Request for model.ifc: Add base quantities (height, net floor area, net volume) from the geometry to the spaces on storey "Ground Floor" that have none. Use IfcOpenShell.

First a look at what the model holds.

```python
import ifcopenshell
import ifcopenshell.util.element
import ifcopenshell.util.unit

model = ifcopenshell.open("model.ifc")
print(model.schema)
for unit_type in ("LENGTHUNIT", "AREAUNIT", "VOLUMEUNIT"):
    print(unit_type, ifcopenshell.util.unit.calculate_unit_scale(model, unit_type))
storey = next(s for s in model.by_type("IfcBuildingStorey") if s.Name == "Ground Floor")
spaces = [e for e in ifcopenshell.util.element.get_decomposition(storey) if e.is_a("IfcSpace")]
for e in sorted(spaces, key=lambda e: e.id()):
    print(e.id(), e.is_a(), e.Name, list(ifcopenshell.util.element.get_psets(e, qtos_only=True)), sep=" | ")
```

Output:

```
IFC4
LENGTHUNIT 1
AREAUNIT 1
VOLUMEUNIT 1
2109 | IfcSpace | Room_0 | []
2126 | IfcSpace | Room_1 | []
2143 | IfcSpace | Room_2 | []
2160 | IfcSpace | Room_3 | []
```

```python
import ifcopenshell
import ifcopenshell.api.pset
import ifcopenshell.geom
import ifcopenshell.util.element
import ifcopenshell.util.shape
import ifcopenshell.util.unit

model = ifcopenshell.open("model.ifc")
unit_scale = ifcopenshell.util.unit.calculate_unit_scale(model)
area_scale = ifcopenshell.util.unit.calculate_unit_scale(model, "AREAUNIT")
volume_scale = ifcopenshell.util.unit.calculate_unit_scale(model, "VOLUMEUNIT")
settings = ifcopenshell.geom.settings()

storey = next(s for s in model.by_type("IfcBuildingStorey") if s.Name == "Ground Floor")
spaces = [e for e in ifcopenshell.util.element.get_decomposition(storey) if e.is_a("IfcSpace")]

for e in sorted(spaces, key=lambda e: e.id()):
    if ifcopenshell.util.element.get_psets(e, qtos_only=True, should_inherit=False):
        continue
    # Geometry comes back in metres, in the element's own axes.
    shape = ifcopenshell.geom.create_shape(settings, e)
    values = {
        "Height": ifcopenshell.util.shape.get_z(shape.geometry) / unit_scale,
        "NetFloorArea": ifcopenshell.util.shape.get_footprint_area(shape.geometry) / area_scale,
        "NetVolume": ifcopenshell.util.shape.get_volume(shape.geometry) / volume_scale,
    }
    qto = ifcopenshell.api.pset.add_qto(model, product=e, name="Qto_SpaceBaseQuantities")
    ifcopenshell.api.pset.edit_qto(model, qto=qto, properties=values)
    print(e.id(), {k: round(v, 3) for k, v in values.items()})

model.write("model_rev.ifc")
```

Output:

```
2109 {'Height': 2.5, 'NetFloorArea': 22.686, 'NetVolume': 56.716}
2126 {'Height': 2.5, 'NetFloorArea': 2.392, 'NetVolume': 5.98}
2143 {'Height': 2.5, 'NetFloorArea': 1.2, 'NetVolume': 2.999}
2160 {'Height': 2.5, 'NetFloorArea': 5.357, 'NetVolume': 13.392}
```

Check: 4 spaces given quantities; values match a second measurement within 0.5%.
